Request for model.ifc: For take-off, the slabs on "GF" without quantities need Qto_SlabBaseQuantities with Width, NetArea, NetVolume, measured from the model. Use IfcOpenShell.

First a look at what the model holds.

```python
import ifcopenshell
import ifcopenshell.util.element
import ifcopenshell.util.unit

model = ifcopenshell.open("model.ifc")
print(model.schema)
for unit_type in ("LENGTHUNIT", "AREAUNIT", "VOLUMEUNIT"):
    print(unit_type, ifcopenshell.util.unit.calculate_unit_scale(model, unit_type))
storey = next(s for s in model.by_type("IfcBuildingStorey") if s.Name == "GF")
slabs = [e for e in ifcopenshell.util.element.get_decomposition(storey) if e.is_a("IfcSlab")]
for e in sorted(slabs, key=lambda e: e.id()):
    print(e.id(), e.is_a(), e.Name, list(ifcopenshell.util.element.get_psets(e, qtos_only=True)), sep=" | ")
```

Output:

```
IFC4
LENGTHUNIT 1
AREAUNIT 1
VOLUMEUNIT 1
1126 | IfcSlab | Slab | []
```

```python
import ifcopenshell
import ifcopenshell.api.pset
import ifcopenshell.geom
import ifcopenshell.util.element
import ifcopenshell.util.shape
import ifcopenshell.util.unit

model = ifcopenshell.open("model.ifc")
unit_scale = ifcopenshell.util.unit.calculate_unit_scale(model)
area_scale = ifcopenshell.util.unit.calculate_unit_scale(model, "AREAUNIT")
volume_scale = ifcopenshell.util.unit.calculate_unit_scale(model, "VOLUMEUNIT")
settings = ifcopenshell.geom.settings()

storey = next(s for s in model.by_type("IfcBuildingStorey") if s.Name == "GF")
slabs = [e for e in ifcopenshell.util.element.get_decomposition(storey) if e.is_a("IfcSlab")]

for e in sorted(slabs, key=lambda e: e.id()):
    if ifcopenshell.util.element.get_psets(e, qtos_only=True, should_inherit=False):
        continue
    # Geometry comes back in metres, in the element's own axes.
    shape = ifcopenshell.geom.create_shape(settings, e)
    values = {
        "Width": ifcopenshell.util.shape.get_z(shape.geometry) / unit_scale,
        "NetArea": ifcopenshell.util.shape.get_footprint_area(shape.geometry) / area_scale,
        "NetVolume": ifcopenshell.util.shape.get_volume(shape.geometry) / volume_scale,
    }
    qto = ifcopenshell.api.pset.add_qto(model, product=e, name="Qto_SlabBaseQuantities")
    ifcopenshell.api.pset.edit_qto(model, qto=qto, properties=values)
    print(e.id(), {k: round(v, 3) for k, v in values.items()})

model.write("model_updated.ifc")
```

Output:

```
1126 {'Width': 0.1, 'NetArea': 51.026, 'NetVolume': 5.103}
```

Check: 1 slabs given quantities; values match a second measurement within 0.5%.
